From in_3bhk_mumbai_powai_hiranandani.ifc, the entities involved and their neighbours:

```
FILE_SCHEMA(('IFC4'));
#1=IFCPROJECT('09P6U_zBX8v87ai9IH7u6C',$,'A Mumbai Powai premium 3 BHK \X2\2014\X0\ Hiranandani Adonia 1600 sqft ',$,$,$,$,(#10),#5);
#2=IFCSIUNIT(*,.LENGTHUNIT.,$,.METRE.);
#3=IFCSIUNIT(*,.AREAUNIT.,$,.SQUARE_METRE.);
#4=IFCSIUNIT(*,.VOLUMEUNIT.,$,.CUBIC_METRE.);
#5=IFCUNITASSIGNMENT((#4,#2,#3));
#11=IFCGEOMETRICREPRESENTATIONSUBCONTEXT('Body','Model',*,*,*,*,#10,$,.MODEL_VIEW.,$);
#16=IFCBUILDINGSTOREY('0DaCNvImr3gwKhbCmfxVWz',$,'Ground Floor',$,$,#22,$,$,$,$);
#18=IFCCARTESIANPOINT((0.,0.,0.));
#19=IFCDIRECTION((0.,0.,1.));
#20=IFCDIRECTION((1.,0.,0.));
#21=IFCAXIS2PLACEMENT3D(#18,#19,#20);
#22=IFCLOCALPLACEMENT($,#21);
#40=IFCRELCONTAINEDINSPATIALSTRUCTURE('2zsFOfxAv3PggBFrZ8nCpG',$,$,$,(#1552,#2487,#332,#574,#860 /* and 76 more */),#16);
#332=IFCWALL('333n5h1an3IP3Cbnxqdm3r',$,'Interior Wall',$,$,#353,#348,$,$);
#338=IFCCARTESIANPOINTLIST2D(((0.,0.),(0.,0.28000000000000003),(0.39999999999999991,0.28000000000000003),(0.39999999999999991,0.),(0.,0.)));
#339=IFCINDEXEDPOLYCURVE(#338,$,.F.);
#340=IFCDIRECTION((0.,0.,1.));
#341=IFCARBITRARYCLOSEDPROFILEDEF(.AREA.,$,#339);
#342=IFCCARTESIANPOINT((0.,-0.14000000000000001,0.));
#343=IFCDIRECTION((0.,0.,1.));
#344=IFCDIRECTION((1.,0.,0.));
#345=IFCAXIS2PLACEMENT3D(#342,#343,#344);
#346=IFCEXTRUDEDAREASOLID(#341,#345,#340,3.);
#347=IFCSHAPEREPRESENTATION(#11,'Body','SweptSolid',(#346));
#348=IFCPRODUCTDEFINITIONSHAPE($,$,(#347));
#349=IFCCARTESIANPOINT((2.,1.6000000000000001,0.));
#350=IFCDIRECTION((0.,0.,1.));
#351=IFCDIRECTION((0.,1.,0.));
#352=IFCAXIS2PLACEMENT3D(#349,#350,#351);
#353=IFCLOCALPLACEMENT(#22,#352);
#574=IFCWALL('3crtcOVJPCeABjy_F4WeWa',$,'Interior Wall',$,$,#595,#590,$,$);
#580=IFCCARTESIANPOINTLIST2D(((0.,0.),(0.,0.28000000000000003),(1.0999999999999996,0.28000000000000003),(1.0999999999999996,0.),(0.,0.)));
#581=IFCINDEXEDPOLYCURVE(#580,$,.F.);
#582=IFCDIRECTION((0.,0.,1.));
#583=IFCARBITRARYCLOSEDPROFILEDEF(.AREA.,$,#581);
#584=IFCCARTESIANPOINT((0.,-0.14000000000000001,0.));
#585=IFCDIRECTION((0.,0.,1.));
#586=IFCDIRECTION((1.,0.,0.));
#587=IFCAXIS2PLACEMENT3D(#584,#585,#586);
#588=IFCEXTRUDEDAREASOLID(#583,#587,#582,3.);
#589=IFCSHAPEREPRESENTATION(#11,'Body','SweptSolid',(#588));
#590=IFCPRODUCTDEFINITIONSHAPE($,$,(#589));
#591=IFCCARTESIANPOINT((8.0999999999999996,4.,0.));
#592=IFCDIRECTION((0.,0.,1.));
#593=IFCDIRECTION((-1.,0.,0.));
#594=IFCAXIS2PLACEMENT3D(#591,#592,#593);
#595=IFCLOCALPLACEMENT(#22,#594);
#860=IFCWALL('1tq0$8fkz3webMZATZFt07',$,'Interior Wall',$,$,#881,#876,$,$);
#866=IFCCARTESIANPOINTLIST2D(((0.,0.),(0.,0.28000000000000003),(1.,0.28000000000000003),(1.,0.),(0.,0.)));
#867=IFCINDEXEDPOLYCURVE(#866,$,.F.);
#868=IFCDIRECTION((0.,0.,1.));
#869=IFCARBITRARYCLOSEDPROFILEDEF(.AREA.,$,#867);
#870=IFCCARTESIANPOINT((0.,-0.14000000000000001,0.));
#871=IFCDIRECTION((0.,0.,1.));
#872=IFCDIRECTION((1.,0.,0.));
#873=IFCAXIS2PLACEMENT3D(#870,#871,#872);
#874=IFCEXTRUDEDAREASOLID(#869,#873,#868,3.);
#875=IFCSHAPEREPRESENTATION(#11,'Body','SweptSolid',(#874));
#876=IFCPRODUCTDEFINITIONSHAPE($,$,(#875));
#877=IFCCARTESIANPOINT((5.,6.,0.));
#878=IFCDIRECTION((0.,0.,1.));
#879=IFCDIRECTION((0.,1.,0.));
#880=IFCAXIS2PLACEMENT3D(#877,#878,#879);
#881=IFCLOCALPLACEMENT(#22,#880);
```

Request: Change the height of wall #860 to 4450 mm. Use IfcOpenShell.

```python
import ifcopenshell
import ifcopenshell.geom
import ifcopenshell.util.representation
import ifcopenshell.util.shape
import ifcopenshell.util.unit

model = ifcopenshell.open("in_3bhk_mumbai_powai_hiranandani.ifc")
unit_scale = ifcopenshell.util.unit.calculate_unit_scale(model)
settings = ifcopenshell.geom.settings()


def volume(element):
    """Net volume in cubic metres, openings subtracted."""
    shape = ifcopenshell.geom.create_shape(settings, element)
    return ifcopenshell.util.shape.get_volume(shape.geometry)


wall = model.by_guid("1tq0$8fkz3webMZATZFt07")
before = volume(wall)

body = ifcopenshell.util.representation.get_representation(wall, "Model", "Body")
solid = body.Items[0]
old_height = solid.Depth
solid.Depth = 4.45 / unit_scale
after = volume(wall)

print(f"height {old_height:g} -> {solid.Depth:g}, volume {before:.3f} -> {after:.3f} m3")

model.write("in_3bhk_mumbai_powai_hiranandani-out.ifc")
```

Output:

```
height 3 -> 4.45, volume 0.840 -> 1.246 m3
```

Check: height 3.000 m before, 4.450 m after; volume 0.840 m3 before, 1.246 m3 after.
